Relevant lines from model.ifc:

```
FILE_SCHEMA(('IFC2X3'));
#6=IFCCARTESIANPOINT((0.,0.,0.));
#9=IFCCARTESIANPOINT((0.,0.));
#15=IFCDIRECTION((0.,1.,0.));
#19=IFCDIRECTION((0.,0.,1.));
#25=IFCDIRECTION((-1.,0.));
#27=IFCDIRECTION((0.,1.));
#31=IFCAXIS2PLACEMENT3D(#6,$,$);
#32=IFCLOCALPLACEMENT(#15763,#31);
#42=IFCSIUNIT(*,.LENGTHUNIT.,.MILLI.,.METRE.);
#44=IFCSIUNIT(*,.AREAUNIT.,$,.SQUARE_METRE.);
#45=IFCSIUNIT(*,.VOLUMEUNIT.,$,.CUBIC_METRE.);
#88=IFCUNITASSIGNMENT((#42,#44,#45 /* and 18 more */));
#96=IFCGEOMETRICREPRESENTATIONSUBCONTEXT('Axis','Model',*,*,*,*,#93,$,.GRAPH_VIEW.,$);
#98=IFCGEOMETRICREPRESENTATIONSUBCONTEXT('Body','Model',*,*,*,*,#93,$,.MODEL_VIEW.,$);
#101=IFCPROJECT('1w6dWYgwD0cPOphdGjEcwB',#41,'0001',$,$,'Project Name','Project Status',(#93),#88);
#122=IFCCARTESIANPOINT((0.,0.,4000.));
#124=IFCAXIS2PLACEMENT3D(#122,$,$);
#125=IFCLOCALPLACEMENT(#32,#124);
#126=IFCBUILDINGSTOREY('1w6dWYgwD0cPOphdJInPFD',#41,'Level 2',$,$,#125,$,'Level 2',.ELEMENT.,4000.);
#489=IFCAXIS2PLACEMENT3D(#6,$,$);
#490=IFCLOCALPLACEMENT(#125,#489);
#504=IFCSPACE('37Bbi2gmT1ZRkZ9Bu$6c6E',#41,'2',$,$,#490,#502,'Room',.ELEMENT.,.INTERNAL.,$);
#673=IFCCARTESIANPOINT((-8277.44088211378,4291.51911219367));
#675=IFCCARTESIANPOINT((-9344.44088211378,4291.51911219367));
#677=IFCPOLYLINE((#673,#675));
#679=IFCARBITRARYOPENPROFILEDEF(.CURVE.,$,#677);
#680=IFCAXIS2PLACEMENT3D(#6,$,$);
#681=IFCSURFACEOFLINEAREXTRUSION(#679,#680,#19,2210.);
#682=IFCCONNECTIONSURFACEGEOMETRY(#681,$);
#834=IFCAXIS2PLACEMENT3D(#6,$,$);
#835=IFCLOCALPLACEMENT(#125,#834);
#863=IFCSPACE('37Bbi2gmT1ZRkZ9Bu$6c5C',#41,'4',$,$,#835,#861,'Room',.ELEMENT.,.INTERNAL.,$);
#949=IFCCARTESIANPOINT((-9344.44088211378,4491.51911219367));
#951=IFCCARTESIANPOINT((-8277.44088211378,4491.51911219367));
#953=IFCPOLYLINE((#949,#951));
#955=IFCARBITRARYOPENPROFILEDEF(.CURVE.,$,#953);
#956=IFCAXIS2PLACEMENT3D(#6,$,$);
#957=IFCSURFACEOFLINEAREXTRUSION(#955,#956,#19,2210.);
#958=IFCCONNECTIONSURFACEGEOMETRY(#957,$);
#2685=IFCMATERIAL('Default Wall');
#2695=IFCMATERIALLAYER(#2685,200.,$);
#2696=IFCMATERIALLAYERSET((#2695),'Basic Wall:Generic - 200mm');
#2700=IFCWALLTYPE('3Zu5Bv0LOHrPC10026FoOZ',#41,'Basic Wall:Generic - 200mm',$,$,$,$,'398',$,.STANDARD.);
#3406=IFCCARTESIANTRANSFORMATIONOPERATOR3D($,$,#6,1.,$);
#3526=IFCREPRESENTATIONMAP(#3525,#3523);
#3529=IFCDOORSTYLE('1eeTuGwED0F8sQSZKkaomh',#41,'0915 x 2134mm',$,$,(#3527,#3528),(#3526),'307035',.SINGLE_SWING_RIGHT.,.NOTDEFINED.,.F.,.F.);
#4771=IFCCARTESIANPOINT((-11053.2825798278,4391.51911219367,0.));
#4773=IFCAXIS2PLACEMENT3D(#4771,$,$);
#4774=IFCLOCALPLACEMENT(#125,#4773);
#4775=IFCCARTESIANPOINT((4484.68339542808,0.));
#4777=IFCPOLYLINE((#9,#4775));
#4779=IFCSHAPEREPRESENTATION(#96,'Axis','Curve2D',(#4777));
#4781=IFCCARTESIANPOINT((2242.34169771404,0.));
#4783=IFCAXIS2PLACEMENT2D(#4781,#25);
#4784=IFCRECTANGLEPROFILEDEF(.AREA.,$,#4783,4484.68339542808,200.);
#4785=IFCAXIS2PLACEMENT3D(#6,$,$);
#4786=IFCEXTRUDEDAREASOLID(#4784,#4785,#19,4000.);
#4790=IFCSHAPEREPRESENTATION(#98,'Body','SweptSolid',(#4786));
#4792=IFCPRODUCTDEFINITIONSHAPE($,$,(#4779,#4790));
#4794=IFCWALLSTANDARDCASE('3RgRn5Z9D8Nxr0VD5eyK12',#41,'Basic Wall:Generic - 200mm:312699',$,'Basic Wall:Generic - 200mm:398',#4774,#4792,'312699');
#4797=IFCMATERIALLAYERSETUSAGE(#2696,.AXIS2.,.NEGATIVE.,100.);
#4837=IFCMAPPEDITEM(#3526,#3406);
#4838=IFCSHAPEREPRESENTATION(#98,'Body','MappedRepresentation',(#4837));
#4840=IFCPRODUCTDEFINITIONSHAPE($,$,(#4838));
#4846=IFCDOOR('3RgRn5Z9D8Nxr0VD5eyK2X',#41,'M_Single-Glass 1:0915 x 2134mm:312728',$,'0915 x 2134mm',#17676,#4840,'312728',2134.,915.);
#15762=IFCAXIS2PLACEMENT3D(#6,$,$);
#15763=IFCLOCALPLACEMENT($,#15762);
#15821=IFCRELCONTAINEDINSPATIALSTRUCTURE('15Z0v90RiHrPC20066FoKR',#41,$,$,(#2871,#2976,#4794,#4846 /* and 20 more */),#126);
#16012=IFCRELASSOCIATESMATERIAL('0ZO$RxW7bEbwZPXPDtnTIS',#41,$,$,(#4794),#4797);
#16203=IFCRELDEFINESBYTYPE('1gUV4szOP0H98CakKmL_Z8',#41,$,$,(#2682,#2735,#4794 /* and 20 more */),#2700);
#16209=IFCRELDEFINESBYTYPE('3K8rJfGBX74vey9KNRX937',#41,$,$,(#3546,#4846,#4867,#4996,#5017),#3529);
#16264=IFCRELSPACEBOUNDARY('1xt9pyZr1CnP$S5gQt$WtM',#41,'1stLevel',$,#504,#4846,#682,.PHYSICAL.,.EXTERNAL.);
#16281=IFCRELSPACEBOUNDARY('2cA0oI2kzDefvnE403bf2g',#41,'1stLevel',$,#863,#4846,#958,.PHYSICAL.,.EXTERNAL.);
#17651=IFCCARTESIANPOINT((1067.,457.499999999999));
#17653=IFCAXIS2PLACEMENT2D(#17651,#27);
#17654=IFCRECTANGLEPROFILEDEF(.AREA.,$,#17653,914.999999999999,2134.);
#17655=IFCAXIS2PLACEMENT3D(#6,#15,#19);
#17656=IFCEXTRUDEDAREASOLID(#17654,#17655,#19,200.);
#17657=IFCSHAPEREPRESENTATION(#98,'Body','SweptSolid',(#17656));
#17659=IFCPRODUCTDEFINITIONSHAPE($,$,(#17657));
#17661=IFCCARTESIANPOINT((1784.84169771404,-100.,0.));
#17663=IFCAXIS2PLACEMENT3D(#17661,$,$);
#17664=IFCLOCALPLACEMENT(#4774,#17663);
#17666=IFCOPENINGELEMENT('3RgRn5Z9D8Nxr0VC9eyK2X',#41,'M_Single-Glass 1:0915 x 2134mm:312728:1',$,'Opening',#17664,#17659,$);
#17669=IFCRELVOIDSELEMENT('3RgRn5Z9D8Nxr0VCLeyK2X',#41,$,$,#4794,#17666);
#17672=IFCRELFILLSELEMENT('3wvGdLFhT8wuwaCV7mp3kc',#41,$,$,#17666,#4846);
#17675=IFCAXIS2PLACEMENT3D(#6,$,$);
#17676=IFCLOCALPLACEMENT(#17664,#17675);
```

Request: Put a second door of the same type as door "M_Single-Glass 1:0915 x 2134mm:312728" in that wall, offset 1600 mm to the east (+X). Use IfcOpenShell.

```python
import numpy as np
import ifcopenshell
import ifcopenshell.api.feature
import ifcopenshell.api.geometry
import ifcopenshell.api.root
import ifcopenshell.geom
import ifcopenshell.util.element
import ifcopenshell.util.placement
import ifcopenshell.util.shape
import ifcopenshell.util.unit

model = ifcopenshell.open("model.ifc")
unit_scale = ifcopenshell.util.unit.calculate_unit_scale(model)
settings = ifcopenshell.geom.settings()


def volume(element):
    """Net volume in cubic metres, openings subtracted."""
    shape = ifcopenshell.geom.create_shape(settings, element)
    return ifcopenshell.util.shape.get_volume(shape.geometry)


def reuse_history(source, copy):
    """copy_class also copies each property set's owner history, people and application; keep the originals."""
    for rel in copy.IsDefinedBy:
        if rel.is_a("IfcRelDefinesByProperties") and (history := rel.RelatingPropertyDefinition.OwnerHistory):
            rel.RelatingPropertyDefinition.OwnerHistory = source.OwnerHistory
            ifcopenshell.util.element.remove_deep2(model, history)


door = model.by_guid("3RgRn5Z9D8Nxr0VD5eyK2X")
opening = door.FillsVoids[0].RelatingOpeningElement
wall = opening.VoidsElements[0].RelatingBuildingElement
before = volume(wall)
shift = ifcopenshell.util.placement.get_local_placement(wall.ObjectPlacement)[:3, 0] * 1.6 / unit_scale

# copy_class copies the void relationship, type, container and properties, but no geometry.
new_opening = ifcopenshell.api.root.copy_class(model, product=opening)
new_opening.Representation = ifcopenshell.util.element.copy_deep(
    model, opening.Representation, exclude=["IfcGeometricRepresentationContext", "IfcRepresentationMap"]
)
new_opening.Name = "M_Single-Glass 1:0915 x 2134mm"
new_door = ifcopenshell.api.root.copy_class(model, product=door)
new_door.Representation = ifcopenshell.util.element.copy_deep(
    model, door.Representation, exclude=["IfcGeometricRepresentationContext", "IfcRepresentationMap"]
)
new_door.Name = "M_Single-Glass 1:0915 x 2134mm"
new_door.Tag = None
reuse_history(door, new_door)
fills = ifcopenshell.api.feature.add_filling(model, opening=new_opening, element=new_door)
fills.OwnerHistory = new_door.OwnerHistory  # required in IFC2X3

for old, new in ((opening, new_opening), (door, new_door)):
    matrix = ifcopenshell.util.placement.get_local_placement(old.ObjectPlacement)
    matrix[:3, 3] += shift
    ifcopenshell.api.geometry.edit_object_placement(model, product=new, matrix=matrix, is_si=False)

# The copied space boundaries still share their surfaces with the original.
for rel in new_door.ProvidesBoundaries:
    if rel.ConnectionGeometry:
        rel.ConnectionGeometry = ifcopenshell.util.element.copy_deep(model, rel.ConnectionGeometry)

# Space boundary surfaces are stored in each space's coordinates; move them too.
for rel in new_door.ProvidesBoundaries:
    if not rel.ConnectionGeometry:
        continue
    surface = rel.ConnectionGeometry.SurfaceOnRelatingElement
    space_matrix = ifcopenshell.util.placement.get_local_placement(rel.RelatingSpace.ObjectPlacement)
    point = np.array(surface.Position.Location.Coordinates) + space_matrix[:3, :3].T @ shift
    surface.Position = model.createIfcAxis2Placement3D(
        model.createIfcCartesianPoint(point.tolist()), surface.Position.Axis, surface.Position.RefDirection
    )

after = volume(wall)

print(f"wall volume {before:.3f} -> {after:.3f} m3")

model.write("model-out.ifc")
```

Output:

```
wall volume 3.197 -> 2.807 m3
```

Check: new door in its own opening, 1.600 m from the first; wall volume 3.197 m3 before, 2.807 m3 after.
